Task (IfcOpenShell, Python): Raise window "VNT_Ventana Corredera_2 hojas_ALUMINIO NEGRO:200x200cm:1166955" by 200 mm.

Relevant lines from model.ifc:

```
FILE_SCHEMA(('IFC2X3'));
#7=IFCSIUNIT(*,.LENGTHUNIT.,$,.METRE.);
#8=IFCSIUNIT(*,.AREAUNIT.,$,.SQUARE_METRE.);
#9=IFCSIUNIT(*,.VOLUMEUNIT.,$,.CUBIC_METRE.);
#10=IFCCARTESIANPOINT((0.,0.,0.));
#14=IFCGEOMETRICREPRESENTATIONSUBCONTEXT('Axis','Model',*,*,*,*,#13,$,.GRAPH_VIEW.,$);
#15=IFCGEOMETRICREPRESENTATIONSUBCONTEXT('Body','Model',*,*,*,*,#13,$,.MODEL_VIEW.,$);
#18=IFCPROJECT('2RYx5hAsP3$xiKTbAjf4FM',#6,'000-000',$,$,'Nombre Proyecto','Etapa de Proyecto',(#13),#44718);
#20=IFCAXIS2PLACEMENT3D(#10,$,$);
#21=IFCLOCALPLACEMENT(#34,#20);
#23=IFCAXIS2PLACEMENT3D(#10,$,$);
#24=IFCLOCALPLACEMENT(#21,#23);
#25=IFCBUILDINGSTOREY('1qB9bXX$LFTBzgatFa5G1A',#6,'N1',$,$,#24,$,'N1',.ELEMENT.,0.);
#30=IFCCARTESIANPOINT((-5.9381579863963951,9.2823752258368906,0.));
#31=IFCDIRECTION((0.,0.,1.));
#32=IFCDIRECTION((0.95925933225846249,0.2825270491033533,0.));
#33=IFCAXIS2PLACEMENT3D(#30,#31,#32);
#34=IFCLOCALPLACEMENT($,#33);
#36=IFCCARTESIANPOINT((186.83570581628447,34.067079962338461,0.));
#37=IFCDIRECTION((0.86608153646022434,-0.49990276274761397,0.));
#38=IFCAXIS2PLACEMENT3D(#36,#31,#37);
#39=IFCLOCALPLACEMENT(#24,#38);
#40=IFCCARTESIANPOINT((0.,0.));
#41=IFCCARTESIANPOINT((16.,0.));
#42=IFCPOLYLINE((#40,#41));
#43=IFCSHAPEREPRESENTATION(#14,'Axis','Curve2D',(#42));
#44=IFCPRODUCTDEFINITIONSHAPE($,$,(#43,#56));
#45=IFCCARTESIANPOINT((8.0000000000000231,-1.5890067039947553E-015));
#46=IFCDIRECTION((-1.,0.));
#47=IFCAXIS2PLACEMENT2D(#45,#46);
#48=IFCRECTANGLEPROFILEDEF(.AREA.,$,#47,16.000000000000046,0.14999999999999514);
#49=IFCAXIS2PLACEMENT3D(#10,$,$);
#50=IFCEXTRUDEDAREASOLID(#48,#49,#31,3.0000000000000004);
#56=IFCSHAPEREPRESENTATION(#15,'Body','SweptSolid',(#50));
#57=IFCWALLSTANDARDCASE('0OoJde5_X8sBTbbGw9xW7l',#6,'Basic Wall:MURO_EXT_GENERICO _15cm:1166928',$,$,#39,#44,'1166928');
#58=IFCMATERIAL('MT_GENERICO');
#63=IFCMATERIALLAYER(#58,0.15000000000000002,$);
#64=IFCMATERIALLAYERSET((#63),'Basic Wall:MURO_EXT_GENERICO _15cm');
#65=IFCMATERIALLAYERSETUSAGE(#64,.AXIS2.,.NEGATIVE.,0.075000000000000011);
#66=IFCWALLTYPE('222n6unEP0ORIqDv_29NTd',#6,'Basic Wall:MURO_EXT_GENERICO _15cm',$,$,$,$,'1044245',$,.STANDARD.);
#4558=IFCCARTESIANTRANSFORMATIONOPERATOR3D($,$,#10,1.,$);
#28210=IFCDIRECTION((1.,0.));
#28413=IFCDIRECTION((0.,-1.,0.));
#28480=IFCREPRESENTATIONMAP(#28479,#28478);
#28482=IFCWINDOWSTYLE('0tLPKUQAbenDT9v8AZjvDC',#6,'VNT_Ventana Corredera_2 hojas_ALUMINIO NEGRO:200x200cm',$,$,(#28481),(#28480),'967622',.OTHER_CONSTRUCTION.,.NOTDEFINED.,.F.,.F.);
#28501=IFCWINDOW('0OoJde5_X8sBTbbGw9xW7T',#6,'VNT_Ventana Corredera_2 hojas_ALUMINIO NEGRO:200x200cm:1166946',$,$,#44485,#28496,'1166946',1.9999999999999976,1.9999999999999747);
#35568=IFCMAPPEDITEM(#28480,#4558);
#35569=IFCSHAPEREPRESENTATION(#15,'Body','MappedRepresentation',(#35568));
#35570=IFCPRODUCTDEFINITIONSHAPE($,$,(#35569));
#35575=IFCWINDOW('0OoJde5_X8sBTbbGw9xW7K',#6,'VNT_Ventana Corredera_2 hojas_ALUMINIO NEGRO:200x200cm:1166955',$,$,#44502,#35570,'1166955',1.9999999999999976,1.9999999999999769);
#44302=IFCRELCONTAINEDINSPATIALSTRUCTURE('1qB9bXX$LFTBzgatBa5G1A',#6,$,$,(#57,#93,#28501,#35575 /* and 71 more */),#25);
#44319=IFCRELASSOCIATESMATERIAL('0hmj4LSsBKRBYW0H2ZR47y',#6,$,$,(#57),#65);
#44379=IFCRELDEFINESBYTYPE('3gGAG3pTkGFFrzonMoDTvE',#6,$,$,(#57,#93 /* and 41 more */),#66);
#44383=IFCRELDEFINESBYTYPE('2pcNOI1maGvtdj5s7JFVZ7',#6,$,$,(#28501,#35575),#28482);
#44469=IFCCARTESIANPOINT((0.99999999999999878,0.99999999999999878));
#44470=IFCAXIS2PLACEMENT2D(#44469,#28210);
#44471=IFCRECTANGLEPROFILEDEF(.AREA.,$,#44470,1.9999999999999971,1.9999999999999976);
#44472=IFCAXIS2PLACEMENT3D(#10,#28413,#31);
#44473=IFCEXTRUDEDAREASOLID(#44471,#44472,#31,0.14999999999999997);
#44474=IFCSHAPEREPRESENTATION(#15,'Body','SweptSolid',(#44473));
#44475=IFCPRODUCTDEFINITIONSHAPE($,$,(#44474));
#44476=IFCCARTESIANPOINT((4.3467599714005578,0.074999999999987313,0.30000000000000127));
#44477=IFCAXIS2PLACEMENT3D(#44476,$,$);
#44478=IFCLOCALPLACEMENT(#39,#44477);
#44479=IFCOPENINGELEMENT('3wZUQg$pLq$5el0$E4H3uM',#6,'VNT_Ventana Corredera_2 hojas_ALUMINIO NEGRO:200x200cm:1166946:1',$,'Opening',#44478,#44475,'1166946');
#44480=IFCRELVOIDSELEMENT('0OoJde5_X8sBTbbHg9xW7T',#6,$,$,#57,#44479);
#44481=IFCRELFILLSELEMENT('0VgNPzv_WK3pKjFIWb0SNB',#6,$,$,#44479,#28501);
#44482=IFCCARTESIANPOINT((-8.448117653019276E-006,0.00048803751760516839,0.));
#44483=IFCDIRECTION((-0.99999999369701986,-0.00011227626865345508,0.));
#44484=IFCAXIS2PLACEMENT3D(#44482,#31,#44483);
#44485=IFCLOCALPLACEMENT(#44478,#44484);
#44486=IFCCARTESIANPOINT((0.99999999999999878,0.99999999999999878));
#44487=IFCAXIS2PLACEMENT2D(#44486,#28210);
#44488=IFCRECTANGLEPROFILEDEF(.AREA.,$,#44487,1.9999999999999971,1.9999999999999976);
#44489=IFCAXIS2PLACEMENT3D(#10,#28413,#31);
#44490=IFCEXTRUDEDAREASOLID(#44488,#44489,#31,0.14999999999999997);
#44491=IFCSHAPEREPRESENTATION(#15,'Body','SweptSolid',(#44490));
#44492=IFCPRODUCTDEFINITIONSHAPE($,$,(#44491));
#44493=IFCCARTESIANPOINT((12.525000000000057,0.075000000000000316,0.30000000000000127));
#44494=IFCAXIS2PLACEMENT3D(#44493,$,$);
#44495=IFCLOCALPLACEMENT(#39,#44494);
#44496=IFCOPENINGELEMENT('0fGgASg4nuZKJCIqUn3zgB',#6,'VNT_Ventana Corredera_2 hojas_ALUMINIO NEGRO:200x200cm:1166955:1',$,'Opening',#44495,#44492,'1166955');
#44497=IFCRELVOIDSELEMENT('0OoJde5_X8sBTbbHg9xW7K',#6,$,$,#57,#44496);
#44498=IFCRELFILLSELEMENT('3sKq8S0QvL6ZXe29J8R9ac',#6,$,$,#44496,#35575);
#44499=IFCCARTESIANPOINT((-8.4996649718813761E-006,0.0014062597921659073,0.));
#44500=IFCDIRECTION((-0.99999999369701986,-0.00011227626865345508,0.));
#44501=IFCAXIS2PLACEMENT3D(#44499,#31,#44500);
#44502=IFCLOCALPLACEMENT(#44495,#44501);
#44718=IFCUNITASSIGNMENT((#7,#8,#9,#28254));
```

```python
import numpy as np
import ifcopenshell
import ifcopenshell.api.geometry
import ifcopenshell.util.placement
import ifcopenshell.util.unit

model = ifcopenshell.open("model.ifc")
unit_scale = ifcopenshell.util.unit.calculate_unit_scale(model)

window = model.by_id(35575)
opening = window.FillsVoids[0].RelatingOpeningElement
dz = 0.2 / unit_scale

shift = np.array([0.0, 0.0, dz])
# The window is placed relative to its opening, so it follows when the opening moves.
matrix = ifcopenshell.util.placement.get_local_placement(opening.ObjectPlacement)
matrix[:3, 3] += shift
ifcopenshell.api.geometry.edit_object_placement(
    model, product=opening, matrix=matrix, is_si=False, should_transform_children=True
)

print(f"moved by {dz * unit_scale:+.3f} m")

model.write("model_updated.ifc")
```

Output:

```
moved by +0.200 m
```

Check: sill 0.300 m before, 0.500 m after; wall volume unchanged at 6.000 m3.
